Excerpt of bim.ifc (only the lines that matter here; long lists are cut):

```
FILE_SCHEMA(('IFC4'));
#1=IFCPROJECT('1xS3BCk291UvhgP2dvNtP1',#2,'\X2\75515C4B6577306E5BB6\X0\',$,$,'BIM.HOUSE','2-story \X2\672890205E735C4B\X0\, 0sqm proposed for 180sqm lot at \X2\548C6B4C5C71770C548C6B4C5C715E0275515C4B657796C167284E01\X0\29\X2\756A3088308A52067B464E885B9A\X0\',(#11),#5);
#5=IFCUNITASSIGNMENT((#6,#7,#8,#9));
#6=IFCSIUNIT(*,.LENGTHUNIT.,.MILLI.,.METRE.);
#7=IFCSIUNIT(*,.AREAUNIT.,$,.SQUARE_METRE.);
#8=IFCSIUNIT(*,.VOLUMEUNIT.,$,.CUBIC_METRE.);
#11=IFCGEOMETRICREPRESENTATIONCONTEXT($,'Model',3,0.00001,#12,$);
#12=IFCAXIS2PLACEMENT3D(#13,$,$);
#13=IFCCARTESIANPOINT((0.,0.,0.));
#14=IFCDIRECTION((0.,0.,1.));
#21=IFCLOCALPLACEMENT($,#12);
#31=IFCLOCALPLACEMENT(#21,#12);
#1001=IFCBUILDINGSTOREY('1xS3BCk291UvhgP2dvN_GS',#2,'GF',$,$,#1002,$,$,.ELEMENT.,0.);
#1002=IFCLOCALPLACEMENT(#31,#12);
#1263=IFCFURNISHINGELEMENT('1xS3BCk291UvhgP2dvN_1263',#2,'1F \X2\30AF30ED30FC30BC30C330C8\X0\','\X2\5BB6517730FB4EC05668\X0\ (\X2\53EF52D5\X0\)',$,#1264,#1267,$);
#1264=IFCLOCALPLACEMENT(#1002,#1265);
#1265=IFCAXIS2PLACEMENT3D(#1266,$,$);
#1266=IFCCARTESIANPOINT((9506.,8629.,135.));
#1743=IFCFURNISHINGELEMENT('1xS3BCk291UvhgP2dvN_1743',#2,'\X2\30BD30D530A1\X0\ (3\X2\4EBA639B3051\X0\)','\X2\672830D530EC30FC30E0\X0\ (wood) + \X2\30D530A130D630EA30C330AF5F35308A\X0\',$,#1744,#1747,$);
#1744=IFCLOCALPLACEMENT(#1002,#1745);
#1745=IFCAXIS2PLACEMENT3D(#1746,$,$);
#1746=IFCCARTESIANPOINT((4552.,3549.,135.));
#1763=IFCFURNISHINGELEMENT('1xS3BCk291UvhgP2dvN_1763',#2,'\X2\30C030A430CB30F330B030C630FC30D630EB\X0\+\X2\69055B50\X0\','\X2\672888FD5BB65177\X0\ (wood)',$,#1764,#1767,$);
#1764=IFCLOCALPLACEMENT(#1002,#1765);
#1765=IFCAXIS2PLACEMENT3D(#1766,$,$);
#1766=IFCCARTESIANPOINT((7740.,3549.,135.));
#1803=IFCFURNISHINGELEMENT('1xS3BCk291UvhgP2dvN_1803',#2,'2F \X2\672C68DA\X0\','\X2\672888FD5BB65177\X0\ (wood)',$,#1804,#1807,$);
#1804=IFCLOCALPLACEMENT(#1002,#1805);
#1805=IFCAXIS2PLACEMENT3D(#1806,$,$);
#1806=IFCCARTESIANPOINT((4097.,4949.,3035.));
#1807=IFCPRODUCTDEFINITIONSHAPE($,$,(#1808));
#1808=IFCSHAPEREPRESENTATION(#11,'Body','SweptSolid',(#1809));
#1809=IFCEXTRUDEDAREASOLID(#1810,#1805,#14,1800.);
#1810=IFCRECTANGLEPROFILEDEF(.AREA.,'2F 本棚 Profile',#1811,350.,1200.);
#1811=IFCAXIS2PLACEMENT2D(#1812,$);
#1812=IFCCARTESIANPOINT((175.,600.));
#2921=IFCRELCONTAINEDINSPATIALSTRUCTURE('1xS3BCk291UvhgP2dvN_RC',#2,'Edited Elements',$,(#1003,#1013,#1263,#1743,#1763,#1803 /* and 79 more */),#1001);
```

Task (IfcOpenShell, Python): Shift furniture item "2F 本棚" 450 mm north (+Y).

```python
import ifcopenshell
import ifcopenshell.api.geometry
import ifcopenshell.util.placement

model = ifcopenshell.open("bim.ifc")

item = model.by_guid("1xS3BCk291UvhgP2dvN_1803")
matrix = ifcopenshell.util.placement.get_local_placement(item.ObjectPlacement)
matrix[1, 3] += 450.0
ifcopenshell.api.geometry.edit_object_placement(model, product=item, matrix=matrix, is_si=False)

print(ifcopenshell.util.placement.get_local_placement(item.ObjectPlacement).round(3) + 0.0)

model.write("bim_edited.ifc")
```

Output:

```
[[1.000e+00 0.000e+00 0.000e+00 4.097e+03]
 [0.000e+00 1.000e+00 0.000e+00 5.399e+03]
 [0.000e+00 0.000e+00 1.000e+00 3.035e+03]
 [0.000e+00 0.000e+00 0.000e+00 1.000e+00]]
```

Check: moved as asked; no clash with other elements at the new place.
